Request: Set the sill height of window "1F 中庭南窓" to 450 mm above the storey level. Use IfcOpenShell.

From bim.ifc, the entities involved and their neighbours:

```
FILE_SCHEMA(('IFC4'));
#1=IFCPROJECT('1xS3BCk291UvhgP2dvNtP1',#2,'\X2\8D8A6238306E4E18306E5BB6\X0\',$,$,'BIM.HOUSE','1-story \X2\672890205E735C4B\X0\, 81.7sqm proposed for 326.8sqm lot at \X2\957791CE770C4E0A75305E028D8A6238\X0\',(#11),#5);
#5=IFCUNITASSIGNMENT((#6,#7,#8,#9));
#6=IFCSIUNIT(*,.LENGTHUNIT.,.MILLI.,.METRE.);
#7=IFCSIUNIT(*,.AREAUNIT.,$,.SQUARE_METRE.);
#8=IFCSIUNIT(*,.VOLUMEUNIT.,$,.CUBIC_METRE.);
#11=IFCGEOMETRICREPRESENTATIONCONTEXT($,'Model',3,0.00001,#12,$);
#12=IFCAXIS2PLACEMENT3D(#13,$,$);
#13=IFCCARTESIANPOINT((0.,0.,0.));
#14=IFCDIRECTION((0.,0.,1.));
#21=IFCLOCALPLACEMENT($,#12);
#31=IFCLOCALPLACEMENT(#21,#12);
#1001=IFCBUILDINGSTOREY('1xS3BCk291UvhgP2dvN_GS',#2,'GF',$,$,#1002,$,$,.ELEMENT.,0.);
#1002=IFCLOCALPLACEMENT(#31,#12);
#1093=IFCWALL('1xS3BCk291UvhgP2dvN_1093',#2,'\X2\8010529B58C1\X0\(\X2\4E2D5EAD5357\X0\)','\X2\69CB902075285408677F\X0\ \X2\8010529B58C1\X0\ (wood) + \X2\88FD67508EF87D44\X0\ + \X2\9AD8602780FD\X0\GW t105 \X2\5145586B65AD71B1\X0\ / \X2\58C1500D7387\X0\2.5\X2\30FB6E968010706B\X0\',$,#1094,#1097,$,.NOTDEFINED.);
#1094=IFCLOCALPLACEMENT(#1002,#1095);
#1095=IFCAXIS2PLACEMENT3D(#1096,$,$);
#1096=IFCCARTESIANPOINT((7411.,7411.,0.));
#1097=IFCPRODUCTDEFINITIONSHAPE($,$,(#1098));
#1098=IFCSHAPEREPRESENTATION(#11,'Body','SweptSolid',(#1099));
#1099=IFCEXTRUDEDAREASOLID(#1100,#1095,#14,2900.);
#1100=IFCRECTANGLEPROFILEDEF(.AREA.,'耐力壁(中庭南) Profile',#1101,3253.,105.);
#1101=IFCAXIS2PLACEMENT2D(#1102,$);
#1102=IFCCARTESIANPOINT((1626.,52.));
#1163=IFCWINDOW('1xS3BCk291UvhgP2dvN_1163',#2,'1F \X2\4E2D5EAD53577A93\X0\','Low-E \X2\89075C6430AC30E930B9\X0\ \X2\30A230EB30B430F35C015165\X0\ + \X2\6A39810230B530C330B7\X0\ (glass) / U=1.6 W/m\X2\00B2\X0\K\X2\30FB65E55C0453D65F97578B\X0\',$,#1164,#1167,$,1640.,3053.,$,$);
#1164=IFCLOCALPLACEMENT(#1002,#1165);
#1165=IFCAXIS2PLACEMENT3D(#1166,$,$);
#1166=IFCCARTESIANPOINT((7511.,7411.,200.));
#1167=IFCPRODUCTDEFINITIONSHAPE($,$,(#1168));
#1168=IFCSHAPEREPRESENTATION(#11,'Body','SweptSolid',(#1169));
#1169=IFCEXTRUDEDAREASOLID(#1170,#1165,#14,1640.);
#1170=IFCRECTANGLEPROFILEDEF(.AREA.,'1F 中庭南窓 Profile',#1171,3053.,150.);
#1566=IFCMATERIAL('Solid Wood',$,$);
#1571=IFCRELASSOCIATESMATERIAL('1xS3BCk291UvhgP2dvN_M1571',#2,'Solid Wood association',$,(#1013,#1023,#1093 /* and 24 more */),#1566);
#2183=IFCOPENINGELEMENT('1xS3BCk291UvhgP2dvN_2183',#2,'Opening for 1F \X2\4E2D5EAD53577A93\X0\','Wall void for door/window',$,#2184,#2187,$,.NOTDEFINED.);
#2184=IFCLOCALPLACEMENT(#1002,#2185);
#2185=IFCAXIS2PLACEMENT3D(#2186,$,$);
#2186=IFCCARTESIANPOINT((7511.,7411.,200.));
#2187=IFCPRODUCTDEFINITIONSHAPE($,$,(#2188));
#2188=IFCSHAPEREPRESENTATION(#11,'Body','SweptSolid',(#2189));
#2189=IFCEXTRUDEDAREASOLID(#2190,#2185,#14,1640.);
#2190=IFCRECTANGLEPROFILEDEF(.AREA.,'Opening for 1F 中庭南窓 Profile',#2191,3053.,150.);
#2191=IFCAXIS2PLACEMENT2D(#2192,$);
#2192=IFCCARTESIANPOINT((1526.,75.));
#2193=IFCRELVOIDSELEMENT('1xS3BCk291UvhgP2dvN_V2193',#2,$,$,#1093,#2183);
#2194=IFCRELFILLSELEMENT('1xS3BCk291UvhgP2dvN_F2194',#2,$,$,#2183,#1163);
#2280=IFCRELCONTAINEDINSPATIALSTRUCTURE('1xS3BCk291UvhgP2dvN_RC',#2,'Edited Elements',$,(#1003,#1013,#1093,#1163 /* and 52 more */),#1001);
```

```python
import numpy as np
import ifcopenshell
import ifcopenshell.api.geometry
import ifcopenshell.geom
import ifcopenshell.util.element
import ifcopenshell.util.placement
import ifcopenshell.util.shape
import ifcopenshell.util.unit

model = ifcopenshell.open("bim.ifc")
unit_scale = ifcopenshell.util.unit.calculate_unit_scale(model)

window = model.by_id(1163)
opening = window.FillsVoids[0].RelatingOpeningElement
storey = ifcopenshell.util.element.get_container(window, ifc_class="IfcBuildingStorey")
level = ifcopenshell.util.placement.get_local_placement(storey.ObjectPlacement)[2, 3]

# The opening's origin need not be at the sill, so measure its lowest point.
shape = ifcopenshell.geom.create_shape(ifcopenshell.geom.settings(), opening)
bottom = ifcopenshell.util.shape.get_shape_bottom_elevation(shape, shape.geometry) / unit_scale
dz = level + 0.45 / unit_scale - bottom

shift = np.array([0.0, 0.0, dz])
# The window is not placed relative to its opening, so move both.
for product in (opening, window):
    matrix = ifcopenshell.util.placement.get_local_placement(product.ObjectPlacement)
    matrix[:3, 3] += shift
    ifcopenshell.api.geometry.edit_object_placement(model, product=product, matrix=matrix, is_si=False)

print(f"moved by {dz * unit_scale:+.3f} m")

model.write("bim_rev.ifc")
```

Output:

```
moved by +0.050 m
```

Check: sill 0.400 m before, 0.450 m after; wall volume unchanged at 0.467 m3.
